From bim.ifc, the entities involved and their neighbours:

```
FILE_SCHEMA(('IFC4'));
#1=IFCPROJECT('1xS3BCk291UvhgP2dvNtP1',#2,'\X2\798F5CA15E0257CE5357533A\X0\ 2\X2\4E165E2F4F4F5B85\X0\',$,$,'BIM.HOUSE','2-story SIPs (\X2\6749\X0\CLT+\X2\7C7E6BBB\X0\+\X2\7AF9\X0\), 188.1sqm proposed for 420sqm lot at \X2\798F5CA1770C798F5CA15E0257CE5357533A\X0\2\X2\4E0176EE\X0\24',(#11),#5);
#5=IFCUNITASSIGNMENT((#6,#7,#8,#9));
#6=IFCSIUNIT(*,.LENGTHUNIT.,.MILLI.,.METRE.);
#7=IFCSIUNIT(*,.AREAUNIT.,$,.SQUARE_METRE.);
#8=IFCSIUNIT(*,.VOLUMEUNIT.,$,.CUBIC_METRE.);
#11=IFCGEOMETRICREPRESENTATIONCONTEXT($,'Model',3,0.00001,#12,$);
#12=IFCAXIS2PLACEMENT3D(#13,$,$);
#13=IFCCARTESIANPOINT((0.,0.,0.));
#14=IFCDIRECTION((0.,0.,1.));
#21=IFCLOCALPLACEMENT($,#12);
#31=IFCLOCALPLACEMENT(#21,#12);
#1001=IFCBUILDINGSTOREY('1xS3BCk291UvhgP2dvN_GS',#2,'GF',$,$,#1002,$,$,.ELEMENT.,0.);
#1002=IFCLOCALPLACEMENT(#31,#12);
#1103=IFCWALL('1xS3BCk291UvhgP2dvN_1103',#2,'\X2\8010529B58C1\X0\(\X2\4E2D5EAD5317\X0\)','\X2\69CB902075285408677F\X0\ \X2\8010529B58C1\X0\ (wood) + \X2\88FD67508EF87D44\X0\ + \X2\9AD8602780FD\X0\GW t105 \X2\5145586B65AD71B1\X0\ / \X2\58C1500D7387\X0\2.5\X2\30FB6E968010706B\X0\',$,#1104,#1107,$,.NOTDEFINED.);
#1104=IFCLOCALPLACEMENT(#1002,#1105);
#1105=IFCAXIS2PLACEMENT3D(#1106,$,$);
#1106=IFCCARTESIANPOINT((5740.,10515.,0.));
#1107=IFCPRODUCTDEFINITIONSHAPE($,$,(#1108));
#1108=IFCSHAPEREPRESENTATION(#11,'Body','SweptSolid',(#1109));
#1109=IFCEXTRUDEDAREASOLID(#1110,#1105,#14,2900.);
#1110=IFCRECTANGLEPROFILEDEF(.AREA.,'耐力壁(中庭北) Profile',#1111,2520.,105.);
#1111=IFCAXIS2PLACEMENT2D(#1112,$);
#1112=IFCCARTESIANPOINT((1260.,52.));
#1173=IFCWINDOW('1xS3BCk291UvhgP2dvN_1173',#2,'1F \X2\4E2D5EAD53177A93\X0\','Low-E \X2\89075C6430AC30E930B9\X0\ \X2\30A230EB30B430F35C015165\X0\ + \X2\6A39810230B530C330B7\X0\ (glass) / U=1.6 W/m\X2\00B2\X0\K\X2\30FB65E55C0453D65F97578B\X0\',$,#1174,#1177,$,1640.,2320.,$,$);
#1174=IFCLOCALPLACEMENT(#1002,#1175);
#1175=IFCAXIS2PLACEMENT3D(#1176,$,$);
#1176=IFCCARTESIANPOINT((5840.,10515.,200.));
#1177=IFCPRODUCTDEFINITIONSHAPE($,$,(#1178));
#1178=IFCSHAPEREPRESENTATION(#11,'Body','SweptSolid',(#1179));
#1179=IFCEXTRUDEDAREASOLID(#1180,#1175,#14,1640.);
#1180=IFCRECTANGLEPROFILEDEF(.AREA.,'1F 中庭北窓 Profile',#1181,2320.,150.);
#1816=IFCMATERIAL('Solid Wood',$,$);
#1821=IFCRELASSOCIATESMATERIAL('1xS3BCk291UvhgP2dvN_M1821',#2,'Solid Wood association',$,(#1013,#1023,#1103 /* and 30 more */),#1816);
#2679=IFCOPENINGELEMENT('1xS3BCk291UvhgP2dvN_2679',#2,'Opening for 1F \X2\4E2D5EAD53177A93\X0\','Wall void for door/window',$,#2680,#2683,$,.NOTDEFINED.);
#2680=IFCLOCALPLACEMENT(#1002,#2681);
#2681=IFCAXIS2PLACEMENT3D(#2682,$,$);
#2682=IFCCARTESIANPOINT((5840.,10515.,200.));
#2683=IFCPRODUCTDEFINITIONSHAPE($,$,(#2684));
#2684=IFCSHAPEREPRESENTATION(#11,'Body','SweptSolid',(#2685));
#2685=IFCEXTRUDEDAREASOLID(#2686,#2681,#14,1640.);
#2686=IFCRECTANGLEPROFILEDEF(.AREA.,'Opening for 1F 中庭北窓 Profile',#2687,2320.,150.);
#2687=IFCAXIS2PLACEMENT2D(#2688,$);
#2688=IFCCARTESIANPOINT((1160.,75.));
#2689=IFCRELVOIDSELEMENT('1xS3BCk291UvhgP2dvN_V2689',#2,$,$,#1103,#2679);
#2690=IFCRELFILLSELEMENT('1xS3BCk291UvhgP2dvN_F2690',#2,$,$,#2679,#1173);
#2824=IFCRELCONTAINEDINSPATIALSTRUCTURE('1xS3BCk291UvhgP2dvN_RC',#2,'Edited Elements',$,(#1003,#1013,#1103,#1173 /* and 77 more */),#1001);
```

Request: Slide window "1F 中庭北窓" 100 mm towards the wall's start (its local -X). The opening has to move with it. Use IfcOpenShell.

```python
import ifcopenshell
import ifcopenshell.api.geometry
import ifcopenshell.util.placement
import ifcopenshell.util.unit

model = ifcopenshell.open("bim.ifc")
unit_scale = ifcopenshell.util.unit.calculate_unit_scale(model)

window = model.by_id(1173)
opening = window.FillsVoids[0].RelatingOpeningElement
wall = opening.VoidsElements[0].RelatingBuildingElement

wall_matrix = ifcopenshell.util.placement.get_local_placement(wall.ObjectPlacement)
shift = wall_matrix[:3, 0] * -0.1 / unit_scale
before = ifcopenshell.util.placement.get_local_placement(window.ObjectPlacement)[:3, 3].copy()

# The window is not placed relative to its opening, so move both.
for product in (opening, window):
    matrix = ifcopenshell.util.placement.get_local_placement(product.ObjectPlacement)
    matrix[:3, 3] += shift
    ifcopenshell.api.geometry.edit_object_placement(model, product=product, matrix=matrix, is_si=False)

after = ifcopenshell.util.placement.get_local_placement(window.ObjectPlacement)[:3, 3]
print("window moved by", (after - before).round(3) + 0.0)

model.write("bim_v2.ifc")
```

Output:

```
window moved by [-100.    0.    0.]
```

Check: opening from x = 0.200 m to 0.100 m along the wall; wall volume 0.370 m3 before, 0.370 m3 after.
